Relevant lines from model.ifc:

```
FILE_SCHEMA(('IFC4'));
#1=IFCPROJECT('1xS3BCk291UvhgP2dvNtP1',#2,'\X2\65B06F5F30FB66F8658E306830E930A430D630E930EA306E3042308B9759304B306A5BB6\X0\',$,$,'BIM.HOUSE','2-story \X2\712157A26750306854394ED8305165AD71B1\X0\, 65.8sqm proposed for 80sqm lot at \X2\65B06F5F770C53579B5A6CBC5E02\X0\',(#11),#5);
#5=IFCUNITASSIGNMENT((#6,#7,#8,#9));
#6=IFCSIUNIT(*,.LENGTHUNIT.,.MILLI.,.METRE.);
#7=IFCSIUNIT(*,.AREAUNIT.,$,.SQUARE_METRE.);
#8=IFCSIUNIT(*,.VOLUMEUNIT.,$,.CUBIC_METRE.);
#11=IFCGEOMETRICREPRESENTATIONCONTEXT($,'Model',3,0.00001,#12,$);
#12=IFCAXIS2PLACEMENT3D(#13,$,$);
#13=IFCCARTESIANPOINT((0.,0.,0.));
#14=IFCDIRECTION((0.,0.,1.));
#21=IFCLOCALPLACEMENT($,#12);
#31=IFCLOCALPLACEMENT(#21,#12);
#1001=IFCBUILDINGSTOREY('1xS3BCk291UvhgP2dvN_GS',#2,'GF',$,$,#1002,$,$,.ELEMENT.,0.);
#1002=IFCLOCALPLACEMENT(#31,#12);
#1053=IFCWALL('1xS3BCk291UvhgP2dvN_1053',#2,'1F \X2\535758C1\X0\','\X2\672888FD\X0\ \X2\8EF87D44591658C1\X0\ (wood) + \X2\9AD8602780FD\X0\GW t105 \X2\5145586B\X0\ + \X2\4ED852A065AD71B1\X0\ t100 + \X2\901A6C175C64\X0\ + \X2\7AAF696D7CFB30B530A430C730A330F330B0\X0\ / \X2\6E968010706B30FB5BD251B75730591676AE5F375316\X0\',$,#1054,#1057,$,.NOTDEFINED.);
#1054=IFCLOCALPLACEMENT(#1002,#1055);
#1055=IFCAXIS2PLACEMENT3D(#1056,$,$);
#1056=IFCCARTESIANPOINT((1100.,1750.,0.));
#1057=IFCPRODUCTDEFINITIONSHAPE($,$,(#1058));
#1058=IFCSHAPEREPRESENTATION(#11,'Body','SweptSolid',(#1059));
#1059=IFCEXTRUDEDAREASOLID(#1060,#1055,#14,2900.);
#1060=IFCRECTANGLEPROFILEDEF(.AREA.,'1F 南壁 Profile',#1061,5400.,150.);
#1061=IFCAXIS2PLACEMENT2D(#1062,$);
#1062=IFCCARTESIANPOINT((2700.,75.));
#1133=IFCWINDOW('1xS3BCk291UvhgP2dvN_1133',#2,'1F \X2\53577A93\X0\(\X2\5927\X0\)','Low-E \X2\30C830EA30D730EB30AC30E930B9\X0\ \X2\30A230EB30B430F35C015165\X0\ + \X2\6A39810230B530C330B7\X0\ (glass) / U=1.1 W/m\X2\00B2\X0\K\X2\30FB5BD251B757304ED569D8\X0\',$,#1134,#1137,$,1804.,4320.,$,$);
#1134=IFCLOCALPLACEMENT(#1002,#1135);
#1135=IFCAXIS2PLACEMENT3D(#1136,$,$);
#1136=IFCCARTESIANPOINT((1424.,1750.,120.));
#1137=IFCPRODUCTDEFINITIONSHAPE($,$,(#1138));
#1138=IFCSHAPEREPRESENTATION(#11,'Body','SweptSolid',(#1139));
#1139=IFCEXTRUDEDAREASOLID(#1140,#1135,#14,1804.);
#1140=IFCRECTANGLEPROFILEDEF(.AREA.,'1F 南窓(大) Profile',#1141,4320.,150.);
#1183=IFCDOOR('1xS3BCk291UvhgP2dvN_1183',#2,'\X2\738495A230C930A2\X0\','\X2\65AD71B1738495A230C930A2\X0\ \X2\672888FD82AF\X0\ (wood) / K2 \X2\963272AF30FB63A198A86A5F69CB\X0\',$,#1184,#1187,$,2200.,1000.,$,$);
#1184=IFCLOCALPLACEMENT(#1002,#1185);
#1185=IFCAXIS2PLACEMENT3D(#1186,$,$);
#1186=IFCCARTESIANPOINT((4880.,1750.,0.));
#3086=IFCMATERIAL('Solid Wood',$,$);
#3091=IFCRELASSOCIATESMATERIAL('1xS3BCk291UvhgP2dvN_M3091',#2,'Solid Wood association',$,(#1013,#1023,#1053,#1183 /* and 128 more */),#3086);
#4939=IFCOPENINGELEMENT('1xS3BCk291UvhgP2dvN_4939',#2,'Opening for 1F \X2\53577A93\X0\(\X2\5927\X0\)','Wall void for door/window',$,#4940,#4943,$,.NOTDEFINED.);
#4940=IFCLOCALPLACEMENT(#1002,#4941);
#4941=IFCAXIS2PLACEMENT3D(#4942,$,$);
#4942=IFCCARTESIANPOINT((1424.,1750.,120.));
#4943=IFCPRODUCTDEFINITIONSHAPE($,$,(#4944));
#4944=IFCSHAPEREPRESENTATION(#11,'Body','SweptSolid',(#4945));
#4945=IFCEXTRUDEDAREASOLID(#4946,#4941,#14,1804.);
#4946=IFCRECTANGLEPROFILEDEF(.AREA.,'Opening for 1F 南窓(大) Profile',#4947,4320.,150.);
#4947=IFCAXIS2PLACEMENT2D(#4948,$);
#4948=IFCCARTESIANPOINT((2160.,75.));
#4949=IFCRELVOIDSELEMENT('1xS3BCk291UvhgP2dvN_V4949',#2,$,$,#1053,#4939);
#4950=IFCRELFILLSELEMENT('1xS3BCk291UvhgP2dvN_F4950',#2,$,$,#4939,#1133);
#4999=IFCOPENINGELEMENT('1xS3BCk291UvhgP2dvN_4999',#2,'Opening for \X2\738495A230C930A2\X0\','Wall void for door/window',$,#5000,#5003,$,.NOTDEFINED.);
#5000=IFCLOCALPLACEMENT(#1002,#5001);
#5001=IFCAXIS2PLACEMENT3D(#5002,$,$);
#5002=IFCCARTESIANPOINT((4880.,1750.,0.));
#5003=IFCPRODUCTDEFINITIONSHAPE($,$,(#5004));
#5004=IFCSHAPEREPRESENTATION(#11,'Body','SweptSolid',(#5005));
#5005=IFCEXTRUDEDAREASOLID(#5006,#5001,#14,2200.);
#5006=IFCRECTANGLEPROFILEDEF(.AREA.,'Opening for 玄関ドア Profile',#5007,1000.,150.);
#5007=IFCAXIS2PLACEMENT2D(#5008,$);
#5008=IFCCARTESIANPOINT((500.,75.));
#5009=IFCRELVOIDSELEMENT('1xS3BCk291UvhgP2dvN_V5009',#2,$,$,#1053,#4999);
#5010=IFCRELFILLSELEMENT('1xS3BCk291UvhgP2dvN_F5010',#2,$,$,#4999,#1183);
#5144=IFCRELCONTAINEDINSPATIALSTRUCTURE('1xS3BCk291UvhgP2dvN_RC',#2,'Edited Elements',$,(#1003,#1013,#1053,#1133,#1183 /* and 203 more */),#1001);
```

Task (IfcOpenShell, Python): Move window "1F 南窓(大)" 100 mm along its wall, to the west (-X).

```python
import ifcopenshell
import ifcopenshell.api.geometry
import ifcopenshell.util.placement
import ifcopenshell.util.unit

model = ifcopenshell.open("model.ifc")
unit_scale = ifcopenshell.util.unit.calculate_unit_scale(model)

window = model.by_guid("1xS3BCk291UvhgP2dvN_1133")
opening = window.FillsVoids[0].RelatingOpeningElement
wall = opening.VoidsElements[0].RelatingBuildingElement

wall_matrix = ifcopenshell.util.placement.get_local_placement(wall.ObjectPlacement)
shift = wall_matrix[:3, 0] * -0.1 / unit_scale
before = ifcopenshell.util.placement.get_local_placement(window.ObjectPlacement)[:3, 3].copy()

# The window is not placed relative to its opening, so move both.
for product in (opening, window):
    matrix = ifcopenshell.util.placement.get_local_placement(product.ObjectPlacement)
    matrix[:3, 3] += shift
    ifcopenshell.api.geometry.edit_object_placement(model, product=product, matrix=matrix, is_si=False)

after = ifcopenshell.util.placement.get_local_placement(window.ObjectPlacement)[:3, 3]
print("window moved by", (after - before).round(3) + 0.0)

model.write("model_rev.ifc")
```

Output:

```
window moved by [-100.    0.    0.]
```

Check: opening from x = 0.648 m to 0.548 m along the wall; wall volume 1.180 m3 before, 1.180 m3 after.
